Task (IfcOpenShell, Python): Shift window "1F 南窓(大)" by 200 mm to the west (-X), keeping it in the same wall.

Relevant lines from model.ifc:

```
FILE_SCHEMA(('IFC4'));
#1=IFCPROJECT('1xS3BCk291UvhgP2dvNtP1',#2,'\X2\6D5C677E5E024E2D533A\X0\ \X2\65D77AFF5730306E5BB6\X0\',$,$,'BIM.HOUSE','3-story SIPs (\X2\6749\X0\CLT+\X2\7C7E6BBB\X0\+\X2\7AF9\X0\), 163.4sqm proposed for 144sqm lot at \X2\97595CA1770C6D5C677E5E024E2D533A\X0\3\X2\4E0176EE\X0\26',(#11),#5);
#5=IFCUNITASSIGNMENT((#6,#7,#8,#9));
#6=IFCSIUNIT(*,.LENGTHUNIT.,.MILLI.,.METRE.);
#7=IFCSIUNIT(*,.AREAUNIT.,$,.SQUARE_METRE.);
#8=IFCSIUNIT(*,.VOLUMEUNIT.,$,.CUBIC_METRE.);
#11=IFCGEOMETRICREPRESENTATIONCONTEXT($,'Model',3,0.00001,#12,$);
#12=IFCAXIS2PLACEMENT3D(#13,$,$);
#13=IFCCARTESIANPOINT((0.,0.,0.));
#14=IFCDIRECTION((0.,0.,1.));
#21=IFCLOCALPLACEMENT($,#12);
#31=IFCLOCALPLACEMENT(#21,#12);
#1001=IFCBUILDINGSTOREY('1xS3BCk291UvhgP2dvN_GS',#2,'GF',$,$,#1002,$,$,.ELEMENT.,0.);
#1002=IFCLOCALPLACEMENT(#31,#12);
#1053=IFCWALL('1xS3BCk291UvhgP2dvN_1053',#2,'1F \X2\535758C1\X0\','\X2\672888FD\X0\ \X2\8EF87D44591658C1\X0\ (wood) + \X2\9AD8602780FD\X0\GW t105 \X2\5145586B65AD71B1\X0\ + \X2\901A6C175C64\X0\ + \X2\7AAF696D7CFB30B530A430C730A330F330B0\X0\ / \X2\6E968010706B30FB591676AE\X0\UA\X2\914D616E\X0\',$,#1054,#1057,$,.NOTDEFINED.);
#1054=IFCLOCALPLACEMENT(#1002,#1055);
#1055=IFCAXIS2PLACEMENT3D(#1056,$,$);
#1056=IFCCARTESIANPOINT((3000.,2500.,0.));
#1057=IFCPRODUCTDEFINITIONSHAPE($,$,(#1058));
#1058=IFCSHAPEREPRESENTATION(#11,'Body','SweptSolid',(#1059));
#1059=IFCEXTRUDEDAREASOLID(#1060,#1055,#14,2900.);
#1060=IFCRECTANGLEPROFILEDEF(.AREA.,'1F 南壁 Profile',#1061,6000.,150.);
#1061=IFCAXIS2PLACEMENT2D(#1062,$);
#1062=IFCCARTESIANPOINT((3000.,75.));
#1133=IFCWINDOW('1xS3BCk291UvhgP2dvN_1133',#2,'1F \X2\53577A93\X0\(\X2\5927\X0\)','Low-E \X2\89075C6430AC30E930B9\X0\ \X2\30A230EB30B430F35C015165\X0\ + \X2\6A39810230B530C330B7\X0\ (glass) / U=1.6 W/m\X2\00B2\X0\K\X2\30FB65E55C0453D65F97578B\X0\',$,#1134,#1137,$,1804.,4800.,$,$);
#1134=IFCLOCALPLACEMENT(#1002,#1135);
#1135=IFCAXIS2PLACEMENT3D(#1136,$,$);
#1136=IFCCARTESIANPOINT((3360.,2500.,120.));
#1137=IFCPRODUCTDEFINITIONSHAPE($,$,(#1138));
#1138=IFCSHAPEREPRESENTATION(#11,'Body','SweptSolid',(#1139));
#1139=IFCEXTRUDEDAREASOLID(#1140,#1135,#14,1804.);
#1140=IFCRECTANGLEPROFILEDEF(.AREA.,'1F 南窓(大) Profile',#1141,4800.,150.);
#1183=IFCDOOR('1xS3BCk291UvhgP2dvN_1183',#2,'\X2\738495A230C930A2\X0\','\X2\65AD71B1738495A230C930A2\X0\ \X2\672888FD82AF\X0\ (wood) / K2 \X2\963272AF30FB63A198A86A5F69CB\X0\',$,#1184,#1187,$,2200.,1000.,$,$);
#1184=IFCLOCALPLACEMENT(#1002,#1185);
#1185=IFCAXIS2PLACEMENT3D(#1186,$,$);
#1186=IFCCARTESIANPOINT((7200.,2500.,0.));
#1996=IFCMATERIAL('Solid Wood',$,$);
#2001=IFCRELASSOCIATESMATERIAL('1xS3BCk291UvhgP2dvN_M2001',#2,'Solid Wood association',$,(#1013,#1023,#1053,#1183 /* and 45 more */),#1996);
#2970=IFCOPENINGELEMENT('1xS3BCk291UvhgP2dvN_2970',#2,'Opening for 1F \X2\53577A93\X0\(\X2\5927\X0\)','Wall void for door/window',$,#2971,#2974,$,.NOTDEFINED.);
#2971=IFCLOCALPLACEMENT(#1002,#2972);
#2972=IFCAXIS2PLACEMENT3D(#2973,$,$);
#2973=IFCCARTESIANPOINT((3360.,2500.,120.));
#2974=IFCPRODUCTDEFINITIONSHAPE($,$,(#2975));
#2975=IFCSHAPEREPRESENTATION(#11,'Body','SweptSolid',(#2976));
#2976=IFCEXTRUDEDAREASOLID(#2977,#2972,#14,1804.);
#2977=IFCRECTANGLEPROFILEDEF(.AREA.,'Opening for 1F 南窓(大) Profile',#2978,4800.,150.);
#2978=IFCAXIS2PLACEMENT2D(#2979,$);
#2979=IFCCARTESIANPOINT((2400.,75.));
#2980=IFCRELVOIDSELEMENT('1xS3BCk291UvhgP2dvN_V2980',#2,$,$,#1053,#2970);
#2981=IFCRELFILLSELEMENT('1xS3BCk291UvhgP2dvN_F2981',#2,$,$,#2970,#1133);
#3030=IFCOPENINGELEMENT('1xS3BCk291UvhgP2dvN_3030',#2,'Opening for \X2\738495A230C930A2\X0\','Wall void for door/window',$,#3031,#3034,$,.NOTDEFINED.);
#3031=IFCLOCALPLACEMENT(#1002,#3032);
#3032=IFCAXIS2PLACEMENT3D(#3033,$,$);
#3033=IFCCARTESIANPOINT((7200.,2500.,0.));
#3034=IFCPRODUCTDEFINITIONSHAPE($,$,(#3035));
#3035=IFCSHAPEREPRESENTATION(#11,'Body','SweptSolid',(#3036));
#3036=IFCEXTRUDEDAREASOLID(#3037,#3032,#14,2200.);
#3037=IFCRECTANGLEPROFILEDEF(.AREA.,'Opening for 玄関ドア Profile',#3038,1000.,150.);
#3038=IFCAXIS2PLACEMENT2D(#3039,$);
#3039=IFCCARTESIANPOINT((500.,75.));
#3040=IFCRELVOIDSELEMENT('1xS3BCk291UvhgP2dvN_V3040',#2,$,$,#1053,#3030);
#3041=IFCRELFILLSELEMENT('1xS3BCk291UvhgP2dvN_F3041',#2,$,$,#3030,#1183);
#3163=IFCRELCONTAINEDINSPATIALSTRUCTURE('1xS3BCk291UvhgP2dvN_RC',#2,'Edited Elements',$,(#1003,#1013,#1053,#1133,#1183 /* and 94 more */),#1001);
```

```python
import ifcopenshell
import ifcopenshell.api.geometry
import ifcopenshell.util.placement

model = ifcopenshell.open("model.ifc")

window = model.by_guid("1xS3BCk291UvhgP2dvN_1133")
opening = window.FillsVoids[0].RelatingOpeningElement
wall = opening.VoidsElements[0].RelatingBuildingElement

wall_matrix = ifcopenshell.util.placement.get_local_placement(wall.ObjectPlacement)
shift = wall_matrix[:3, 0] * -200.0
before = ifcopenshell.util.placement.get_local_placement(window.ObjectPlacement)[:3, 3].copy()

# The window is not placed relative to its opening, so move both.
for product in (opening, window):
    matrix = ifcopenshell.util.placement.get_local_placement(product.ObjectPlacement)
    matrix[:3, 3] += shift
    ifcopenshell.api.geometry.edit_object_placement(model, product=product, matrix=matrix, is_si=False)

after = ifcopenshell.util.placement.get_local_placement(window.ObjectPlacement)[:3, 3]
print("window moved by", (after - before).round(3) + 0.0)

model.write("model_rev.ifc")
```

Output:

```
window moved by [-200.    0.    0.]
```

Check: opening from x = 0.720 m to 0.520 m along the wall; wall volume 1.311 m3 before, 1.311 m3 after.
